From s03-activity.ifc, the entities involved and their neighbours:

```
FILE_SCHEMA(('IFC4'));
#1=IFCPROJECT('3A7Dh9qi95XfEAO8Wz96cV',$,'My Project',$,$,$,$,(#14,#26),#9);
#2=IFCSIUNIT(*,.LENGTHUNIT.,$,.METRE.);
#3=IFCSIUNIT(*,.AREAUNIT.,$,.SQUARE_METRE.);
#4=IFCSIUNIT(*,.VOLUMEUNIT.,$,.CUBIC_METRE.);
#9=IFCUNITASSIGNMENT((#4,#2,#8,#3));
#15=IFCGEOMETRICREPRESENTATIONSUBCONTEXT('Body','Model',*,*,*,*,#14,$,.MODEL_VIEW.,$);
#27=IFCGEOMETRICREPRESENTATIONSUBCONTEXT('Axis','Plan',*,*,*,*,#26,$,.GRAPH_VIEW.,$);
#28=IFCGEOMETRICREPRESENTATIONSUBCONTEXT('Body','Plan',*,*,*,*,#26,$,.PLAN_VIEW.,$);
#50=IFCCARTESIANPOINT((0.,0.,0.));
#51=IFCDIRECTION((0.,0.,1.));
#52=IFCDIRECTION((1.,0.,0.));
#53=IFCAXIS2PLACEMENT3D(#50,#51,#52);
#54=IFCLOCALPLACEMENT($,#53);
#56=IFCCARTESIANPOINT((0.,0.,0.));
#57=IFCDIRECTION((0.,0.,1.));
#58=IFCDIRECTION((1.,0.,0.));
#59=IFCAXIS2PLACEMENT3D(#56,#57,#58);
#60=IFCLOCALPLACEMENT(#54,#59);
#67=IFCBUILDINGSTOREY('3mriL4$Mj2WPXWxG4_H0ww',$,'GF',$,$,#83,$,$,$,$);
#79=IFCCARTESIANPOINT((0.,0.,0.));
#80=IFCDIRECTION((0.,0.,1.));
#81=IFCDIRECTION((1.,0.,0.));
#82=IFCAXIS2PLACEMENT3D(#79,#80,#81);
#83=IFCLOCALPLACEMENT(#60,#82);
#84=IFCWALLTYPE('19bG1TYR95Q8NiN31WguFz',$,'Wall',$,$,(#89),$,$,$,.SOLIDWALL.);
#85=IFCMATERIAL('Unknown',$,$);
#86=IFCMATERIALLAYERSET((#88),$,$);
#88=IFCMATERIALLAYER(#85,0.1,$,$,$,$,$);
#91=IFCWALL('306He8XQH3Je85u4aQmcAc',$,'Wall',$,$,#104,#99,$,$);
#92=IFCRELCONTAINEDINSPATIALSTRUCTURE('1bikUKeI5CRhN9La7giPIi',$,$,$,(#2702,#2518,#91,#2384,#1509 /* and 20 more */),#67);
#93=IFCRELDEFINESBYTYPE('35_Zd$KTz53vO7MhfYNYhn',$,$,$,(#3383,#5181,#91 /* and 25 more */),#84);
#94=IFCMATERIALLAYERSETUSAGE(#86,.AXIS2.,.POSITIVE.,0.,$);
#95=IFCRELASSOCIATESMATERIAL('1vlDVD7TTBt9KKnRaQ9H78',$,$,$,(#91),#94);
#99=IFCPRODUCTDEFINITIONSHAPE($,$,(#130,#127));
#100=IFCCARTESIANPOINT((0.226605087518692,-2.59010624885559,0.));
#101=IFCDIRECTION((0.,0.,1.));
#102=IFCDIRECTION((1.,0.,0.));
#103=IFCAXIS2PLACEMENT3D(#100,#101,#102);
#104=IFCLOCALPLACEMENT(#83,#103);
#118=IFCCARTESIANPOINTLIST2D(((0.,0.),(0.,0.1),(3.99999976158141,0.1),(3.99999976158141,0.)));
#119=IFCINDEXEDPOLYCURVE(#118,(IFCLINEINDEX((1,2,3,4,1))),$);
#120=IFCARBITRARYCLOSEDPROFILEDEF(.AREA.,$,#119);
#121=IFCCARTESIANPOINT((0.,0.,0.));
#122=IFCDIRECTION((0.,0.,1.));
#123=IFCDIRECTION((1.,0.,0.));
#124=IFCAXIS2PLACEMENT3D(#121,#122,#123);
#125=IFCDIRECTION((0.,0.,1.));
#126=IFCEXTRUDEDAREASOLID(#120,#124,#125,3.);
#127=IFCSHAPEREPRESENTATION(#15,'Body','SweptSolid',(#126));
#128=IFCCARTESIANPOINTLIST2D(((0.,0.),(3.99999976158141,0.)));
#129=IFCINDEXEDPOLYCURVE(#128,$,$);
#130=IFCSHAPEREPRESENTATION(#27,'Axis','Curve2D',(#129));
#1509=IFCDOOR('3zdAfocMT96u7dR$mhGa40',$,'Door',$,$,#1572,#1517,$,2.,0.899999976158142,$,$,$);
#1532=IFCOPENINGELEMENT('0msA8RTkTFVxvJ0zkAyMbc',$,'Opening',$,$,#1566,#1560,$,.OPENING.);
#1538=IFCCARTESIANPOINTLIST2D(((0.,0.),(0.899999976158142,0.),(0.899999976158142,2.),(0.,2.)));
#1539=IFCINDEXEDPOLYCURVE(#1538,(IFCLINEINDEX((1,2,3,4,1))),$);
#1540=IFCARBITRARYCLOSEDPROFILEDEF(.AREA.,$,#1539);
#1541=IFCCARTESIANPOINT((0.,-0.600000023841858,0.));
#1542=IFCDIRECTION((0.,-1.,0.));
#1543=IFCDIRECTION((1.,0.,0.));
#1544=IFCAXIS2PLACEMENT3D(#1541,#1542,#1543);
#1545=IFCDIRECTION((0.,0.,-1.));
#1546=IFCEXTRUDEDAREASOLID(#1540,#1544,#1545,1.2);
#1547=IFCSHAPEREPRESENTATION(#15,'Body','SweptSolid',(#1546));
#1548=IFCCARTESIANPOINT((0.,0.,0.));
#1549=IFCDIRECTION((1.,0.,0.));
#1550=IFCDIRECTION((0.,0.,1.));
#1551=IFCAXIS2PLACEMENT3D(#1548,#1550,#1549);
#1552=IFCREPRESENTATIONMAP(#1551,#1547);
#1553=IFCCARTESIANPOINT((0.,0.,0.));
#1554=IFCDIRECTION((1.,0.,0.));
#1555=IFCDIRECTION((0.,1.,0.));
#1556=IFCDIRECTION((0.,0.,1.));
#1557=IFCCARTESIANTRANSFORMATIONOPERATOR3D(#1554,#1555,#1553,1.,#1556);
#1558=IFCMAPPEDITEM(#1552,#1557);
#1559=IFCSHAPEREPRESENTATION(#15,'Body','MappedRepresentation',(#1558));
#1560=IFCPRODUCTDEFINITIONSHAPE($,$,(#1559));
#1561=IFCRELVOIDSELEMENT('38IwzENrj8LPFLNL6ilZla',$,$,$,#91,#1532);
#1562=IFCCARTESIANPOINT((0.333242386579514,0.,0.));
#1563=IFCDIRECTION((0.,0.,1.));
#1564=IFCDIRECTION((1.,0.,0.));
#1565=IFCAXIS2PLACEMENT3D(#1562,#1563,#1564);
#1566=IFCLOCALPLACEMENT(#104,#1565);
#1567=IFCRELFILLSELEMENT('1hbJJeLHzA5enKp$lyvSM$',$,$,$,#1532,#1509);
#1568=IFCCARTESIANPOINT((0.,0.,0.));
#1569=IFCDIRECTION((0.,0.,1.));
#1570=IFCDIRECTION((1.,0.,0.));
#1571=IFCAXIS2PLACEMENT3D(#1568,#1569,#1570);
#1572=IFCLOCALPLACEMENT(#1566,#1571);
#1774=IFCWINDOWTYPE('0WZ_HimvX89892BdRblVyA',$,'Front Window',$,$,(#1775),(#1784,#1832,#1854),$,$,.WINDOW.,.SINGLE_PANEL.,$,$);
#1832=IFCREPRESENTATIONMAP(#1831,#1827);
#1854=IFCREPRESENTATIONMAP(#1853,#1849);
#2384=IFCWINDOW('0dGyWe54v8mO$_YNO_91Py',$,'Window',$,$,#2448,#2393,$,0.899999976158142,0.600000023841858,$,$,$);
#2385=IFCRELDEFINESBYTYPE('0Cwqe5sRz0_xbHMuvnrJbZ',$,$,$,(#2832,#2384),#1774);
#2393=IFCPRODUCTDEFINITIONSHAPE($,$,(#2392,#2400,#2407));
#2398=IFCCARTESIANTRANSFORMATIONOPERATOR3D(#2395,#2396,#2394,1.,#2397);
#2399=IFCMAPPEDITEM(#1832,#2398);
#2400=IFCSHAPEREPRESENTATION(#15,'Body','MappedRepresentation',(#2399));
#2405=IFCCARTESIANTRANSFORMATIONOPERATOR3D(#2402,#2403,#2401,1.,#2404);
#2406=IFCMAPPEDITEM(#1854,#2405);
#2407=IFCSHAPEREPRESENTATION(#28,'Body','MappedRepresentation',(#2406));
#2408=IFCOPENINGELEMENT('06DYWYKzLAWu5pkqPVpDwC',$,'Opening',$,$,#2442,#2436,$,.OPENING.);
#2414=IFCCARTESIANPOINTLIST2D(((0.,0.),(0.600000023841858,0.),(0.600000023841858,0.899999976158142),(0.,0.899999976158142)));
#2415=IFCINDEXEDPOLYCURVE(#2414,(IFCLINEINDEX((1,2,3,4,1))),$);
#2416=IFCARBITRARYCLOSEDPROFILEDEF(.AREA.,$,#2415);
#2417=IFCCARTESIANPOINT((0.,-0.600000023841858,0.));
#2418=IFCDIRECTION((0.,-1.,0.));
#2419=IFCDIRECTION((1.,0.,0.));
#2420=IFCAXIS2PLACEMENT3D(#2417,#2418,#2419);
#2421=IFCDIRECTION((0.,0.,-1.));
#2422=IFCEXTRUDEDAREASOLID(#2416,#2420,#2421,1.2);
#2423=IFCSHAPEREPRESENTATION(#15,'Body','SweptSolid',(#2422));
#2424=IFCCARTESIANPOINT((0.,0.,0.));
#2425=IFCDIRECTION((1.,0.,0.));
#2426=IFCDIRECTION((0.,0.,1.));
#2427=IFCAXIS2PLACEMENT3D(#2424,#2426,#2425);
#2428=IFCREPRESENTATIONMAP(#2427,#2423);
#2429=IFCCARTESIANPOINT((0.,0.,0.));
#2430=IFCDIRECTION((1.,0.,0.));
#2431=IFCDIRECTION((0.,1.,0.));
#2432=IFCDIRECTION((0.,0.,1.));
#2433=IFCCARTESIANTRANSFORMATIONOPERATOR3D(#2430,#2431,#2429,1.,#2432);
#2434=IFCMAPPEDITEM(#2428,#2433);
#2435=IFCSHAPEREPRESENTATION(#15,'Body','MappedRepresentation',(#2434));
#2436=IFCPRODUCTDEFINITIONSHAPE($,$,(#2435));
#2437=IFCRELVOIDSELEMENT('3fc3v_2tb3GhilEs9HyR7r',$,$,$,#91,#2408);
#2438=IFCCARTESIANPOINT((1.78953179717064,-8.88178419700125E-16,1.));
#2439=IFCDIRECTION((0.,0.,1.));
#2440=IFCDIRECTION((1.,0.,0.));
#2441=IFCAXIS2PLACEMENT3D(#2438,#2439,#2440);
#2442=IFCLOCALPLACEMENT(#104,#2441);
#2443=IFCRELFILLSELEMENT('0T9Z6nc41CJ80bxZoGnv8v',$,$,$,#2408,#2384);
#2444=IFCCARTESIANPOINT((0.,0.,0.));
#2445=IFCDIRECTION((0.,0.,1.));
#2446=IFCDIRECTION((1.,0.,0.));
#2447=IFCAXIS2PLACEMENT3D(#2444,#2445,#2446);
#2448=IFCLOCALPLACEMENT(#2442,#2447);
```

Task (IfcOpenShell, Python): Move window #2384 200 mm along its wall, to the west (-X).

```python
import ifcopenshell
import ifcopenshell.api.geometry
import ifcopenshell.util.placement
import ifcopenshell.util.unit

model = ifcopenshell.open("s03-activity.ifc")
unit_scale = ifcopenshell.util.unit.calculate_unit_scale(model)

window = model.by_guid("0dGyWe54v8mO$_YNO_91Py")
opening = window.FillsVoids[0].RelatingOpeningElement
wall = opening.VoidsElements[0].RelatingBuildingElement

wall_matrix = ifcopenshell.util.placement.get_local_placement(wall.ObjectPlacement)
shift = wall_matrix[:3, 0] * -0.2 / unit_scale
before = ifcopenshell.util.placement.get_local_placement(window.ObjectPlacement)[:3, 3].copy()

# The window is placed relative to its opening, so it follows when the opening moves.
matrix = ifcopenshell.util.placement.get_local_placement(opening.ObjectPlacement)
matrix[:3, 3] += shift
ifcopenshell.api.geometry.edit_object_placement(
    model, product=opening, matrix=matrix, is_si=False, should_transform_children=True
)

after = ifcopenshell.util.placement.get_local_placement(window.ObjectPlacement)[:3, 3]
print("window moved by", (after - before).round(3) + 0.0)

model.write("s03-activity-out.ifc")
```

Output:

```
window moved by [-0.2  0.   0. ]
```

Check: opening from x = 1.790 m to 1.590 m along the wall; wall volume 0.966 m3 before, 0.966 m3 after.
